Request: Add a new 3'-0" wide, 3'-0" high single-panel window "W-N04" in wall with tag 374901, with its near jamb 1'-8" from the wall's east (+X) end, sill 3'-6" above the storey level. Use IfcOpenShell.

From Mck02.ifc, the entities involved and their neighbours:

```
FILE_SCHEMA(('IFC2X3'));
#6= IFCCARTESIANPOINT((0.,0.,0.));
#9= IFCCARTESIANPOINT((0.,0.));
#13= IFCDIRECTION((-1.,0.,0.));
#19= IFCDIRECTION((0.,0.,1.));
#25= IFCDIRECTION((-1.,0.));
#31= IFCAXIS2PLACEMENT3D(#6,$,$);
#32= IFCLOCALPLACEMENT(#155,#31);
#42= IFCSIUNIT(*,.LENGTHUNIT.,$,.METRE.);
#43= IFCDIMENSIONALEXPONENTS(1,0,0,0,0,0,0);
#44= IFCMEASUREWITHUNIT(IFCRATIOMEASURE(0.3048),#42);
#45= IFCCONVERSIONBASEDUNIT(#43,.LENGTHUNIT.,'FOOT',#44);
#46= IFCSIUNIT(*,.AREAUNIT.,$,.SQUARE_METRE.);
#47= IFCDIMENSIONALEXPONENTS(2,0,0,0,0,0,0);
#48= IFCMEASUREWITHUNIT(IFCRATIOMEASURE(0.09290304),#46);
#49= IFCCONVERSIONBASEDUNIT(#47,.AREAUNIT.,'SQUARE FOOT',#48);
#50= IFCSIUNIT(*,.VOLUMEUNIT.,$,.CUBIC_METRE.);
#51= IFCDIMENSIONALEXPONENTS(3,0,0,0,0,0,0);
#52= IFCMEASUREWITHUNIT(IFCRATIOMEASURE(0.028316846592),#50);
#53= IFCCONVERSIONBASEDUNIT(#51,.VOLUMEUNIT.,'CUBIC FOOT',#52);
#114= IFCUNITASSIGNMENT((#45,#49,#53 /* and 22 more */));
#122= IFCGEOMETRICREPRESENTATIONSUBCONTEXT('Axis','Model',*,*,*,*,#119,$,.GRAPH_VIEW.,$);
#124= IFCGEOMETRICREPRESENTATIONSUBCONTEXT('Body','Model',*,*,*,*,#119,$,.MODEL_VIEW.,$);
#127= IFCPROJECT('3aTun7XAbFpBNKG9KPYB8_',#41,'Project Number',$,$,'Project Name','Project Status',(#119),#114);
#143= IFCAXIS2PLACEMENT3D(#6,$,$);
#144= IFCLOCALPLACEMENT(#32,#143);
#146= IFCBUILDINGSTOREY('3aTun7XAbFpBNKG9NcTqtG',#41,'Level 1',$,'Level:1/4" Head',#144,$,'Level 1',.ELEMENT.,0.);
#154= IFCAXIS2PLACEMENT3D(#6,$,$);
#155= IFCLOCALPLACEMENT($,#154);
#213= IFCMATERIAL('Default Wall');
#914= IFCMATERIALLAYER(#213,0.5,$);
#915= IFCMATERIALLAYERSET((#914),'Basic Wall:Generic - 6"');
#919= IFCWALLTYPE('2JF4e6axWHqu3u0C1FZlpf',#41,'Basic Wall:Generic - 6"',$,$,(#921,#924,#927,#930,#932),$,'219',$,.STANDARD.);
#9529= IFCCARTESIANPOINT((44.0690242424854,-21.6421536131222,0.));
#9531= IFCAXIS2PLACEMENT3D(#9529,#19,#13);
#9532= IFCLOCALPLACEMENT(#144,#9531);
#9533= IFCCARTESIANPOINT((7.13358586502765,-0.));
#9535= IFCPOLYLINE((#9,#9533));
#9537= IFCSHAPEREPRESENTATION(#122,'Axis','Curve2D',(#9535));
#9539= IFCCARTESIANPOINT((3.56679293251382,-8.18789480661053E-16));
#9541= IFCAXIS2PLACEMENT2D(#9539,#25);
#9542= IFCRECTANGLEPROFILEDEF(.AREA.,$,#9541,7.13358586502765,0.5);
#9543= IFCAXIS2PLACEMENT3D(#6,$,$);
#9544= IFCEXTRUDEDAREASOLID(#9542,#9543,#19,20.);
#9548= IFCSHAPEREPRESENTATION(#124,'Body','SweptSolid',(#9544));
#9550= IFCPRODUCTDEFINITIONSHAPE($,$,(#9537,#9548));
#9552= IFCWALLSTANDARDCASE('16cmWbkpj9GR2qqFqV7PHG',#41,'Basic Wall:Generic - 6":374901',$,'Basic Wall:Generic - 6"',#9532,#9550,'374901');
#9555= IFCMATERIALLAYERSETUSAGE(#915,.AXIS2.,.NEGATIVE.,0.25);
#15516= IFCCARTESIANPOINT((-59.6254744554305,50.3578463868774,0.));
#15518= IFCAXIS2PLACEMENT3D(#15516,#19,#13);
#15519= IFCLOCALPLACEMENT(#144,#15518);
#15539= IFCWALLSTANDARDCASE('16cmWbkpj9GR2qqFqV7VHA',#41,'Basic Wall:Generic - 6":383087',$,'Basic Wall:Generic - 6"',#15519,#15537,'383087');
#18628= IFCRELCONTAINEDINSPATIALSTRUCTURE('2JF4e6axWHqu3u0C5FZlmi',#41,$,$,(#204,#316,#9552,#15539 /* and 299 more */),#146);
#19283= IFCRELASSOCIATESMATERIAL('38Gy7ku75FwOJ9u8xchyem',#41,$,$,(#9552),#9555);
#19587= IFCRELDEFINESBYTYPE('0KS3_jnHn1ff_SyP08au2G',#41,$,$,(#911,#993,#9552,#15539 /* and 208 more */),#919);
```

```python
import numpy as np
import ifcopenshell
import ifcopenshell.api.feature
import ifcopenshell.api.geometry
import ifcopenshell.api.root
import ifcopenshell.api.spatial
import ifcopenshell.api.type
import ifcopenshell.geom
import ifcopenshell.util.element
import ifcopenshell.util.placement
import ifcopenshell.util.representation
import ifcopenshell.util.shape
import ifcopenshell.util.unit

model = ifcopenshell.open("Mck02.ifc")
unit_scale = ifcopenshell.util.unit.calculate_unit_scale(model)
settings = ifcopenshell.geom.settings()


def volume(element):
    """Net volume in cubic metres, openings subtracted."""
    shape = ifcopenshell.geom.create_shape(settings, element)
    return ifcopenshell.util.shape.get_volume(shape.geometry)


wall = model.by_guid("16cmWbkpj9GR2qqFqV7PHG")
storey = ifcopenshell.util.element.get_container(wall, ifc_class="IfcBuildingStorey")
context = ifcopenshell.util.representation.get_context(model, "Model", "Body", "MODEL_VIEW")
before = volume(wall)

width, height, from_end, sill = 0.9144, 0.9144, 0.508, 1.0668  # metres

# The wall runs along its own X axis, and the end named is its -X end.
wall_shape = ifcopenshell.geom.create_shape(settings, wall)
x, y, z = ifcopenshell.util.shape.get_vertices(wall_shape.geometry).T
start = x.min() + from_end
face, thickness = float(y.min()), float(y.max() - y.min())
wall_matrix = ifcopenshell.util.placement.get_local_placement(wall.ObjectPlacement)
level = ifcopenshell.util.placement.get_local_placement(storey.ObjectPlacement)[2, 3]


def in_wall(x, y):
    """Placement at x, y metres in the wall's axes, at sill height."""
    matrix = wall_matrix.copy()
    matrix[:, 3] = wall_matrix @ np.array([x / unit_scale, y / unit_scale, 0.0, 1.0])
    matrix[2, 3] = level + sill / unit_scale
    return matrix


# Opening: a box that overshoots both wall faces by 50 mm.
opening = ifcopenshell.api.root.create_entity(model, ifc_class="IfcOpeningElement")
box = ifcopenshell.api.geometry.add_wall_representation(
    model, context=context, length=width, height=height, thickness=thickness + 0.1
)
ifcopenshell.api.geometry.assign_representation(model, product=opening, representation=box)
ifcopenshell.api.geometry.edit_object_placement(model, product=opening, matrix=in_wall(start, face - 0.05), is_si=False)
ifcopenshell.api.feature.add_feature(model, feature=opening, element=wall)

window = ifcopenshell.api.root.create_entity(model, ifc_class="IfcWindow", name="W-N04")
window.OverallWidth, window.OverallHeight = width / unit_scale, height / unit_scale
body = ifcopenshell.api.geometry.add_window_representation(
    model,
    context=context,
    overall_width=window.OverallWidth,
    overall_height=window.OverallHeight,
    partition_type="SINGLE_PANEL",
)
ifcopenshell.api.geometry.assign_representation(model, product=window, representation=body)
ifcopenshell.api.spatial.assign_container(model, products=[window], relating_structure=storey)
fills = ifcopenshell.api.feature.add_filling(model, opening=opening, element=window)
fills.OwnerHistory = window.OwnerHistory  # required in IFC2X3

# IFC2X3 keeps the operation on the window style.
style = ifcopenshell.api.root.create_entity(model, ifc_class="IfcWindowStyle", name="W-N04")
style.OperationType, style.ConstructionType = "SINGLE_PANEL", "NOTDEFINED"
style.ParameterTakesPrecedence = style.Sizeable = False
ifcopenshell.api.type.assign_type(model, related_objects=[window], relating_type=style)

# Centre the window in the wall's thickness.
ifcopenshell.api.geometry.edit_object_placement(model, product=window, matrix=in_wall(start, face), is_si=False)
window_shape = ifcopenshell.geom.create_shape(settings, window)
depth = ifcopenshell.util.shape.get_vertices(window_shape.geometry)[:, 1]
offset = face + thickness / 2 - (depth.min() + depth.max()) / 2
ifcopenshell.api.geometry.edit_object_placement(model, product=window, matrix=in_wall(start, offset), is_si=False)

after = volume(wall)

print(f"wall volume {before:.3f} -> {after:.3f} m3")

model.write("Mck02_edited.ifc")
```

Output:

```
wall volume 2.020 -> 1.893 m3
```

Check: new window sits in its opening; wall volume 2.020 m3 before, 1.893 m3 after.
